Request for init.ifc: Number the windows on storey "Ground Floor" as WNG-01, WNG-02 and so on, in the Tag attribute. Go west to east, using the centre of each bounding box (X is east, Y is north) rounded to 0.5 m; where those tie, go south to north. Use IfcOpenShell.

First a look at what the model holds.

```python
import ifcopenshell
import ifcopenshell.util.element
import ifcopenshell.util.placement

model = ifcopenshell.open("init.ifc")
print(model.schema)
storey = next(s for s in model.by_type("IfcBuildingStorey") if s.Name == "Ground Floor")
windows = [e for e in ifcopenshell.util.element.get_decomposition(storey) if e.is_a("IfcWindow")]
for e in sorted(windows, key=lambda e: e.id()):
    origin = ifcopenshell.util.placement.get_local_placement(e.ObjectPlacement)[:3, 3]
    print(e.id(), e.Tag, e.Name, origin.round(2) + 0.0, sep=" | ")
```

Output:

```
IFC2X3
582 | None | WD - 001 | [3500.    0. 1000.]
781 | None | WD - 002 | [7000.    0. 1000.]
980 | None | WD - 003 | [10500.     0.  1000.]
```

```python
import ifcopenshell
import ifcopenshell.geom
import ifcopenshell.util.element
import ifcopenshell.util.shape

model = ifcopenshell.open("init.ifc")
settings = ifcopenshell.geom.settings()
settings.set("use-world-coords", True)


def centre(element):
    shape = ifcopenshell.geom.create_shape(settings, element)
    return ifcopenshell.util.shape.get_bbox_centroid(shape.geometry)


storey = next(s for s in model.by_type("IfcBuildingStorey") if s.Name == "Ground Floor")
windows = [e for e in ifcopenshell.util.element.get_decomposition(storey) if e.is_a("IfcWindow")]

# Insertion points can sit at a corner or the storey origin, so sort by the geometry (in metres).
centres = {e: centre(e) for e in windows}
windows.sort(key=lambda e: (round(centres[e][0] / 0.5), centres[e][1]))

for i, e in enumerate(windows, start=1):
    number = f"WNG-{i:02d}"
    e.Tag = number
    print(e.id(), number)

model.write("init_edited.ifc")
```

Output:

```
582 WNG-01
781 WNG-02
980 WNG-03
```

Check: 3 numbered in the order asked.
